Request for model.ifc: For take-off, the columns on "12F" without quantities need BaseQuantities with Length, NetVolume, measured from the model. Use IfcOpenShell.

First a look at what the model holds.

```python
import ifcopenshell
import ifcopenshell.util.element
import ifcopenshell.util.unit

model = ifcopenshell.open("model.ifc")
print(model.schema)
for unit_type in ("LENGTHUNIT", "AREAUNIT", "VOLUMEUNIT"):
    print(unit_type, ifcopenshell.util.unit.calculate_unit_scale(model, unit_type))
storey = next(s for s in model.by_type("IfcBuildingStorey") if s.Name == "12F")
columns = [e for e in ifcopenshell.util.element.get_decomposition(storey) if e.is_a("IfcColumn")]
for e in sorted(columns, key=lambda e: e.id()):
    print(e.id(), e.is_a(), e.Name, list(ifcopenshell.util.element.get_psets(e, qtos_only=True)), sep=" | ")
```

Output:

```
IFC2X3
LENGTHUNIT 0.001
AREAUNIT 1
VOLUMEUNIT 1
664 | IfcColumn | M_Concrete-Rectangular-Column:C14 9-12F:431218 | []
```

```python
import ifcopenshell
import ifcopenshell.api.pset
import ifcopenshell.geom
import ifcopenshell.util.element
import ifcopenshell.util.shape
import ifcopenshell.util.unit

model = ifcopenshell.open("model.ifc")
unit_scale = ifcopenshell.util.unit.calculate_unit_scale(model)
volume_scale = ifcopenshell.util.unit.calculate_unit_scale(model, "VOLUMEUNIT")
settings = ifcopenshell.geom.settings()

storey = next(s for s in model.by_type("IfcBuildingStorey") if s.Name == "12F")
columns = [e for e in ifcopenshell.util.element.get_decomposition(storey) if e.is_a("IfcColumn")]

for e in sorted(columns, key=lambda e: e.id()):
    if ifcopenshell.util.element.get_psets(e, qtos_only=True, should_inherit=False):
        continue
    # Geometry comes back in metres, in the element's own axes.
    shape = ifcopenshell.geom.create_shape(settings, e)
    values = {
        "Length": ifcopenshell.util.shape.get_z(shape.geometry) / unit_scale,
        "NetVolume": ifcopenshell.util.shape.get_volume(shape.geometry) / volume_scale,
    }
    qto = ifcopenshell.api.pset.add_qto(model, product=e, name="BaseQuantities")
    ifcopenshell.api.pset.edit_qto(model, qto=qto, properties=values)
    print(e.id(), {k: round(v, 3) for k, v in values.items()})

model.write("model-out.ifc")
```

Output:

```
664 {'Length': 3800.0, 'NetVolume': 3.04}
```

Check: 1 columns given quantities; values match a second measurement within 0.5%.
